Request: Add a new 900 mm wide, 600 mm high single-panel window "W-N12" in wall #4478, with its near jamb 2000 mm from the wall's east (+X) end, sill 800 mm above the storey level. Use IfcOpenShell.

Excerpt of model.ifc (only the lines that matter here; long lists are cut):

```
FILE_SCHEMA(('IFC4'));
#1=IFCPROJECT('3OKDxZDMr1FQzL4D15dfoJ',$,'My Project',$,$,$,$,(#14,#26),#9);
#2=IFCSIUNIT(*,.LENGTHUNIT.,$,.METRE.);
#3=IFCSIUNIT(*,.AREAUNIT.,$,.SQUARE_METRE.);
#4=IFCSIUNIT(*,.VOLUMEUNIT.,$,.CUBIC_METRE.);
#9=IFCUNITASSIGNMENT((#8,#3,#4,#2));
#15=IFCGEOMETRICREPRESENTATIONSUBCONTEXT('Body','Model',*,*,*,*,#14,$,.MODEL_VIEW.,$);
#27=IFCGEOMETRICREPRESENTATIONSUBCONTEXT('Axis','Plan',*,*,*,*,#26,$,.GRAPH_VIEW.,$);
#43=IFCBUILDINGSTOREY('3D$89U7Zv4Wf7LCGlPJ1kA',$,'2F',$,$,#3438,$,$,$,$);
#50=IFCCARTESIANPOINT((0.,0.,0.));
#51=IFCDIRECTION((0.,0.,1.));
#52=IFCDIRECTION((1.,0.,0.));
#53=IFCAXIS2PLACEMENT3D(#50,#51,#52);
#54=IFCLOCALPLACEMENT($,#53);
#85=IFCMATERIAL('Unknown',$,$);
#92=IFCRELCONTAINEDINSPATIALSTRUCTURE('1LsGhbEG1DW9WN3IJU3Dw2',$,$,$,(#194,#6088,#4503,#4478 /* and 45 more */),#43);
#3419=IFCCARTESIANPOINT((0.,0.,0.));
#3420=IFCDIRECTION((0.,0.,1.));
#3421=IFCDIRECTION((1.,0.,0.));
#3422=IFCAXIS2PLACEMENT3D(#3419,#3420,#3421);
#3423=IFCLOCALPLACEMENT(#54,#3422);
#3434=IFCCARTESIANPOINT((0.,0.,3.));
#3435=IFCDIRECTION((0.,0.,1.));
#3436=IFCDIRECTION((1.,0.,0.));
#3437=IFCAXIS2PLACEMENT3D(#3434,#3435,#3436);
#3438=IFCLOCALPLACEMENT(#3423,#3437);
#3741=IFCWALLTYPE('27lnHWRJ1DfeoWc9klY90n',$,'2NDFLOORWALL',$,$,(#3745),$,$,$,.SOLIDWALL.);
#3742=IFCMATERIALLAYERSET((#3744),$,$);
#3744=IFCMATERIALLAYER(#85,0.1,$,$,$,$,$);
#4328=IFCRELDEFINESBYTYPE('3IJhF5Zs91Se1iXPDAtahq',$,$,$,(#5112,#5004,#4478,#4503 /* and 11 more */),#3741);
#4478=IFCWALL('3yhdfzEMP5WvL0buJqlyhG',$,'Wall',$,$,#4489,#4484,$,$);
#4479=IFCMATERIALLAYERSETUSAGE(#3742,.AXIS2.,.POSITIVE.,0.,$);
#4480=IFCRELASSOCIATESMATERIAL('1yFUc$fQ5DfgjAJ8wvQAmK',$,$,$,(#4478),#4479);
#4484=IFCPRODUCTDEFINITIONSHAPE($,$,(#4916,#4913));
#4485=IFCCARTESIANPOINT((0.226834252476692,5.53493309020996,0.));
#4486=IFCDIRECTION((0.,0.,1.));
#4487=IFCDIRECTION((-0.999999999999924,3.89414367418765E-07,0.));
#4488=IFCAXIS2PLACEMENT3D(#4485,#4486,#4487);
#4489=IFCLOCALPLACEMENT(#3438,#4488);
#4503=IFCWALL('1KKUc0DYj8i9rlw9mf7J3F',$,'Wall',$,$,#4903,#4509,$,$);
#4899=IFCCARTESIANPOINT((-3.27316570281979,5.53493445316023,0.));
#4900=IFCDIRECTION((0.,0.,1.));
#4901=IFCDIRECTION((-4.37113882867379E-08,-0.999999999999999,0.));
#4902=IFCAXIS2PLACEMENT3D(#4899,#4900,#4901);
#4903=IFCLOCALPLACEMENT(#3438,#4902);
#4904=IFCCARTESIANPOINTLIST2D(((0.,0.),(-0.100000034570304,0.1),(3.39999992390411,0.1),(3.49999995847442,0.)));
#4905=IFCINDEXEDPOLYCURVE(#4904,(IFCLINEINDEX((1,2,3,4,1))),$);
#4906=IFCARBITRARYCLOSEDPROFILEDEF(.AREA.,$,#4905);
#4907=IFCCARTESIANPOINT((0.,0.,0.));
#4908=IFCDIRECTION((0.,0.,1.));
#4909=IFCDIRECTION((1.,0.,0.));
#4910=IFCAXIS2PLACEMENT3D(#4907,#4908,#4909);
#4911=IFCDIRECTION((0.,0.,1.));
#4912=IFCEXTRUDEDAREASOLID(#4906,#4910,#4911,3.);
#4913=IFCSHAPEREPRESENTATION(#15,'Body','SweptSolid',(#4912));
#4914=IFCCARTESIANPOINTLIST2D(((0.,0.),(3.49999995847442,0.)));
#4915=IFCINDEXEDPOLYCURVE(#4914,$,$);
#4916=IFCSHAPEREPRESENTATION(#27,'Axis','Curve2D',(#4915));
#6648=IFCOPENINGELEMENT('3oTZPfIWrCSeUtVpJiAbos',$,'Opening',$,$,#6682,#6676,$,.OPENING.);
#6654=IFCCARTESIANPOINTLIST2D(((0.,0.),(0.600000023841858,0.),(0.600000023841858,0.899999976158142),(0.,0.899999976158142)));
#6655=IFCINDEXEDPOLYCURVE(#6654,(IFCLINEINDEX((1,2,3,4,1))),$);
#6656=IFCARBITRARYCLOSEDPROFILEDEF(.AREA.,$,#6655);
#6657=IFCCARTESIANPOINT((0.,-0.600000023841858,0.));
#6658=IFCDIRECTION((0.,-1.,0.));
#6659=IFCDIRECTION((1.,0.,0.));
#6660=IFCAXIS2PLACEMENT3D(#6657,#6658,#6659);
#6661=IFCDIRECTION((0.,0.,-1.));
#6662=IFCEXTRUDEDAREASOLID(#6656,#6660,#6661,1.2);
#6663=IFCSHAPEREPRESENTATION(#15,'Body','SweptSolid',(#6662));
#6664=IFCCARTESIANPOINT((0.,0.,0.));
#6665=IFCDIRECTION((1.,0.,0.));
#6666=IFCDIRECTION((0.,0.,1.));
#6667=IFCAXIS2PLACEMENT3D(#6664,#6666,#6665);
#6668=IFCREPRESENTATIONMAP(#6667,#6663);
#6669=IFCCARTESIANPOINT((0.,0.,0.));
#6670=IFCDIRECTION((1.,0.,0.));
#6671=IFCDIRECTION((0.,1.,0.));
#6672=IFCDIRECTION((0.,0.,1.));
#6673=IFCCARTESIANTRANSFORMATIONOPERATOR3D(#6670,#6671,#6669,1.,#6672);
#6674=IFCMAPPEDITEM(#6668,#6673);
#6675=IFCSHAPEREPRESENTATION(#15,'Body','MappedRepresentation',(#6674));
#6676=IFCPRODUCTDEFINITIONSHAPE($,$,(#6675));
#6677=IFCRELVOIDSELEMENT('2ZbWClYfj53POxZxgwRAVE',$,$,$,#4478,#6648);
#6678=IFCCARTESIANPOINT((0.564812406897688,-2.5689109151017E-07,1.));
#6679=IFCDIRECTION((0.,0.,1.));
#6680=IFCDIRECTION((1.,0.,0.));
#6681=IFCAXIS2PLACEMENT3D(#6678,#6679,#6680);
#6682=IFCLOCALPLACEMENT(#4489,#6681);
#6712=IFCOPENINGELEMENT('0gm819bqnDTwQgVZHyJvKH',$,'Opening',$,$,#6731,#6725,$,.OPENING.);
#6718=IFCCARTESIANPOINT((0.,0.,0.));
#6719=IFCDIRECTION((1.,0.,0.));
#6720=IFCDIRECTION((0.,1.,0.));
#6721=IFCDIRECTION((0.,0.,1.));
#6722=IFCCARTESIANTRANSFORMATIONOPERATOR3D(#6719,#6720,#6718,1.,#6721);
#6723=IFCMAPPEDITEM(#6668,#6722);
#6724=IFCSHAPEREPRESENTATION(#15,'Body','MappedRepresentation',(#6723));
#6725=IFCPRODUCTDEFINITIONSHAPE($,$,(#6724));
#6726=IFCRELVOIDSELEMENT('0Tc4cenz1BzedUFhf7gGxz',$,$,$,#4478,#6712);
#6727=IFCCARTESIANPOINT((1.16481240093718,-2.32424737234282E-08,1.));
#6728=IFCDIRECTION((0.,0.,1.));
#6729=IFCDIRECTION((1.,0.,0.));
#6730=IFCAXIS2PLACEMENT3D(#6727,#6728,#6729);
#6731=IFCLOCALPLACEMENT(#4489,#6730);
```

```python
import numpy as np
import ifcopenshell
import ifcopenshell.api.feature
import ifcopenshell.api.geometry
import ifcopenshell.api.root
import ifcopenshell.api.spatial
import ifcopenshell.geom
import ifcopenshell.util.element
import ifcopenshell.util.placement
import ifcopenshell.util.representation
import ifcopenshell.util.shape
import ifcopenshell.util.unit

model = ifcopenshell.open("model.ifc")
unit_scale = ifcopenshell.util.unit.calculate_unit_scale(model)
settings = ifcopenshell.geom.settings()


def volume(element):
    """Net volume in cubic metres, openings subtracted."""
    shape = ifcopenshell.geom.create_shape(settings, element)
    return ifcopenshell.util.shape.get_volume(shape.geometry)


wall = model.by_guid("3yhdfzEMP5WvL0buJqlyhG")
storey = ifcopenshell.util.element.get_container(wall, ifc_class="IfcBuildingStorey")
context = ifcopenshell.util.representation.get_context(model, "Model", "Body", "MODEL_VIEW")
before = volume(wall)

width, height, from_end, sill = 0.9, 0.6, 2, 0.8  # metres

# The wall runs along its own X axis, and the end named is its -X end.
wall_shape = ifcopenshell.geom.create_shape(settings, wall)
x, y, z = ifcopenshell.util.shape.get_vertices(wall_shape.geometry).T
start = x.min() + from_end
face, thickness = float(y.min()), float(y.max() - y.min())
wall_matrix = ifcopenshell.util.placement.get_local_placement(wall.ObjectPlacement)
level = ifcopenshell.util.placement.get_local_placement(storey.ObjectPlacement)[2, 3]


def in_wall(x, y):
    """Placement at x, y metres in the wall's axes, at sill height."""
    matrix = wall_matrix.copy()
    matrix[:, 3] = wall_matrix @ np.array([x / unit_scale, y / unit_scale, 0.0, 1.0])
    matrix[2, 3] = level + sill / unit_scale
    return matrix


# Opening: a box that overshoots both wall faces by 50 mm.
opening = ifcopenshell.api.root.create_entity(model, ifc_class="IfcOpeningElement", predefined_type="OPENING")
box = ifcopenshell.api.geometry.add_wall_representation(
    model, context=context, length=width, height=height, thickness=thickness + 0.1
)
ifcopenshell.api.geometry.assign_representation(model, product=opening, representation=box)
ifcopenshell.api.geometry.edit_object_placement(model, product=opening, matrix=in_wall(start, face - 0.05), is_si=False)
ifcopenshell.api.feature.add_feature(model, feature=opening, element=wall)

window = ifcopenshell.api.root.create_entity(model, ifc_class="IfcWindow", name="W-N12", predefined_type="WINDOW")
window.OverallWidth, window.OverallHeight = width / unit_scale, height / unit_scale
window.PartitioningType = "SINGLE_PANEL"
body = ifcopenshell.api.geometry.add_window_representation(
    model,
    context=context,
    overall_width=window.OverallWidth,
    overall_height=window.OverallHeight,
    partition_type="SINGLE_PANEL",
)
ifcopenshell.api.geometry.assign_representation(model, product=window, representation=body)
ifcopenshell.api.spatial.assign_container(model, products=[window], relating_structure=storey)
ifcopenshell.api.feature.add_filling(model, opening=opening, element=window)

# Centre the window in the wall's thickness.
ifcopenshell.api.geometry.edit_object_placement(model, product=window, matrix=in_wall(start, face), is_si=False)
window_shape = ifcopenshell.geom.create_shape(settings, window)
depth = ifcopenshell.util.shape.get_vertices(window_shape.geometry)[:, 1]
offset = face + thickness / 2 - (depth.min() + depth.max()) / 2
ifcopenshell.api.geometry.edit_object_placement(model, product=window, matrix=in_wall(start, offset), is_si=False)

after = volume(wall)

print(f"wall volume {before:.3f} -> {after:.3f} m3")

model.write("model-out.ifc")
```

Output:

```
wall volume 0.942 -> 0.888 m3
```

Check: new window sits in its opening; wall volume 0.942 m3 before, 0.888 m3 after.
